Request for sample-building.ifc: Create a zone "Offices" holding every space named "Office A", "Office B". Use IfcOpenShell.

First a look at what the model holds.

```python
import ifcopenshell

model = ifcopenshell.open("sample-building.ifc")
print(model.schema)
seen = {}
for space in model.by_type("IfcSpace"):
    seen[space.LongName] = seen.get(space.LongName, 0) + 1
for name, count in sorted(seen.items(), key=str):
    print(count, "x", name)
print("zones:", [z.Name for z in model.by_type("IfcZone")][:20])
```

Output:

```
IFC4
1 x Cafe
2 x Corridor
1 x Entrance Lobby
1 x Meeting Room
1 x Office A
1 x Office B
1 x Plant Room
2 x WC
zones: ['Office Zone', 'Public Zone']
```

```python
import ifcopenshell
import ifcopenshell.api.group
import ifcopenshell.api.root

model = ifcopenshell.open("sample-building.ifc")

names = {"Office A", "Office B"}
spaces = [s for s in model.by_type("IfcSpace") if s.LongName in names]

zone = ifcopenshell.api.root.create_entity(model, ifc_class="IfcZone", name="Offices")
ifcopenshell.api.group.assign_group(model, products=spaces, group=zone)
print(len(spaces), "spaces in", zone.Name)

model.write("sample-building_updated.ifc")
```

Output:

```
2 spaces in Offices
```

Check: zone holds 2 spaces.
